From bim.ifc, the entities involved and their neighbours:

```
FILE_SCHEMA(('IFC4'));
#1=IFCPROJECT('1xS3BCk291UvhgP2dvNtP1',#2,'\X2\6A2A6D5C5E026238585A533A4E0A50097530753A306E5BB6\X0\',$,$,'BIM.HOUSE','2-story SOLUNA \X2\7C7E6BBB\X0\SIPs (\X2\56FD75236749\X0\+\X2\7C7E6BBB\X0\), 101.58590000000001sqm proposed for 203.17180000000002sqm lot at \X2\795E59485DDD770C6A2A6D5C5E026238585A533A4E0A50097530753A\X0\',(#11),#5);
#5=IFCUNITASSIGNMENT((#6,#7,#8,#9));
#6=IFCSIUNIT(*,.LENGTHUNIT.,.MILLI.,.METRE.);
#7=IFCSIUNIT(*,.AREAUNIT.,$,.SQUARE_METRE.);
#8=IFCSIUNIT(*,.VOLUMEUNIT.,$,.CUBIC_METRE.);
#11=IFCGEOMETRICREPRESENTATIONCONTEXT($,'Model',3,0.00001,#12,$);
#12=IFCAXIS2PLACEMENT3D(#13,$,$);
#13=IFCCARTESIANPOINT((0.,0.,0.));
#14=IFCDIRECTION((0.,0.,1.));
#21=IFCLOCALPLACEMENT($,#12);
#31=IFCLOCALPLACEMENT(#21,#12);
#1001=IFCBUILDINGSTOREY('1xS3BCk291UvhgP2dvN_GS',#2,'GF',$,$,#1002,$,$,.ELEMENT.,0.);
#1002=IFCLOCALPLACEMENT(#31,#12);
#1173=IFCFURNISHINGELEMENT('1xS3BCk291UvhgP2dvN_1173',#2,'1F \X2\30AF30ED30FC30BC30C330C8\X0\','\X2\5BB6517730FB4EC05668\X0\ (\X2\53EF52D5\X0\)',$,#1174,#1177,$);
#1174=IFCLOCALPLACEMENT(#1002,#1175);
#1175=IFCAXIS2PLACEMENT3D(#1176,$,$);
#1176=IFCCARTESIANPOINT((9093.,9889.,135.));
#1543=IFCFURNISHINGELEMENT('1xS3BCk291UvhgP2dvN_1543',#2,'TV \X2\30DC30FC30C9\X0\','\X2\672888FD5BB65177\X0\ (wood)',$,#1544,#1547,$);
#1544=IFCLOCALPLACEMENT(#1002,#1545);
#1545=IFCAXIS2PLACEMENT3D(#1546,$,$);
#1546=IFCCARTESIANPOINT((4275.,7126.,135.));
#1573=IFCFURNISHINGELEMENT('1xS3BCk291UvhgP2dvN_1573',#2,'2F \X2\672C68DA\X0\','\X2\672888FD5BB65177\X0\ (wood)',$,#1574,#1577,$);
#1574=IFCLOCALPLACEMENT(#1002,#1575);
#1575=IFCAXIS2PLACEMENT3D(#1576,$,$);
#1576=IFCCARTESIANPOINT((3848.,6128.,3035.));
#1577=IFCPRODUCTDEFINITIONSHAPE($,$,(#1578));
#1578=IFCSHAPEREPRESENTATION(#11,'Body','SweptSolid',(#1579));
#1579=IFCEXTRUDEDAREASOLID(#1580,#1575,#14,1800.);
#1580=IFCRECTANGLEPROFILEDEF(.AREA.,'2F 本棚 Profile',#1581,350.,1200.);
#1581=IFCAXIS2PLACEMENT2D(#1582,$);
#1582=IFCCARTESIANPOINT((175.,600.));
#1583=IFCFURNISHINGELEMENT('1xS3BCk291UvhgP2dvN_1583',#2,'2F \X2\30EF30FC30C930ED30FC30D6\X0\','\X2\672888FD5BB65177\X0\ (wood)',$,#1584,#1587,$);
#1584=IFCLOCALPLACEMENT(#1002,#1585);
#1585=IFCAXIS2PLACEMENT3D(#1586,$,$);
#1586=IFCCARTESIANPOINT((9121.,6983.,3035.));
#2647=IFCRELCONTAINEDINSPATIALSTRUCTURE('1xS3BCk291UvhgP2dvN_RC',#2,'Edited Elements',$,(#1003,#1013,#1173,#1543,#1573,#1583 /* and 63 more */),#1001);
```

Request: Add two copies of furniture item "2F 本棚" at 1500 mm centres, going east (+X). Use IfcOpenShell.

```python
import numpy as np
import ifcopenshell
import ifcopenshell.api.geometry
import ifcopenshell.api.root
import ifcopenshell.util.element
import ifcopenshell.util.placement
import ifcopenshell.util.unit

model = ifcopenshell.open("bim.ifc")
unit_scale = ifcopenshell.util.unit.calculate_unit_scale(model)


def reuse_history(source, copy):
    """copy_class also copies each property set's owner history, people and application; keep the originals."""
    for rel in copy.IsDefinedBy:
        if rel.is_a("IfcRelDefinesByProperties") and (history := rel.RelatingPropertyDefinition.OwnerHistory):
            rel.RelatingPropertyDefinition.OwnerHistory = source.OwnerHistory
            ifcopenshell.util.element.remove_deep2(model, history)


source = model.by_guid("1xS3BCk291UvhgP2dvN_1573")
base = ifcopenshell.util.placement.get_local_placement(source.ObjectPlacement)
step = np.array([1.0, 0.0, 0.0]) * 1.5 / unit_scale

for i in range(1, 3):
    copy = ifcopenshell.api.root.copy_class(model, product=source)
    copy.Representation = ifcopenshell.util.element.copy_deep(
        model, source.Representation, exclude=["IfcGeometricRepresentationContext", "IfcRepresentationMap"]
    )
    reuse_history(source, copy)
    matrix = base.copy()
    matrix[:3, 3] += i * step
    print("added at", matrix[:3, 3].round(3) + 0.0)
    ifcopenshell.api.geometry.edit_object_placement(model, product=copy, matrix=matrix, is_si=False)

model.write("bim_edited.ifc")
```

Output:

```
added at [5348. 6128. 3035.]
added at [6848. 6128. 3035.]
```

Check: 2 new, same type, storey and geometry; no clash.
